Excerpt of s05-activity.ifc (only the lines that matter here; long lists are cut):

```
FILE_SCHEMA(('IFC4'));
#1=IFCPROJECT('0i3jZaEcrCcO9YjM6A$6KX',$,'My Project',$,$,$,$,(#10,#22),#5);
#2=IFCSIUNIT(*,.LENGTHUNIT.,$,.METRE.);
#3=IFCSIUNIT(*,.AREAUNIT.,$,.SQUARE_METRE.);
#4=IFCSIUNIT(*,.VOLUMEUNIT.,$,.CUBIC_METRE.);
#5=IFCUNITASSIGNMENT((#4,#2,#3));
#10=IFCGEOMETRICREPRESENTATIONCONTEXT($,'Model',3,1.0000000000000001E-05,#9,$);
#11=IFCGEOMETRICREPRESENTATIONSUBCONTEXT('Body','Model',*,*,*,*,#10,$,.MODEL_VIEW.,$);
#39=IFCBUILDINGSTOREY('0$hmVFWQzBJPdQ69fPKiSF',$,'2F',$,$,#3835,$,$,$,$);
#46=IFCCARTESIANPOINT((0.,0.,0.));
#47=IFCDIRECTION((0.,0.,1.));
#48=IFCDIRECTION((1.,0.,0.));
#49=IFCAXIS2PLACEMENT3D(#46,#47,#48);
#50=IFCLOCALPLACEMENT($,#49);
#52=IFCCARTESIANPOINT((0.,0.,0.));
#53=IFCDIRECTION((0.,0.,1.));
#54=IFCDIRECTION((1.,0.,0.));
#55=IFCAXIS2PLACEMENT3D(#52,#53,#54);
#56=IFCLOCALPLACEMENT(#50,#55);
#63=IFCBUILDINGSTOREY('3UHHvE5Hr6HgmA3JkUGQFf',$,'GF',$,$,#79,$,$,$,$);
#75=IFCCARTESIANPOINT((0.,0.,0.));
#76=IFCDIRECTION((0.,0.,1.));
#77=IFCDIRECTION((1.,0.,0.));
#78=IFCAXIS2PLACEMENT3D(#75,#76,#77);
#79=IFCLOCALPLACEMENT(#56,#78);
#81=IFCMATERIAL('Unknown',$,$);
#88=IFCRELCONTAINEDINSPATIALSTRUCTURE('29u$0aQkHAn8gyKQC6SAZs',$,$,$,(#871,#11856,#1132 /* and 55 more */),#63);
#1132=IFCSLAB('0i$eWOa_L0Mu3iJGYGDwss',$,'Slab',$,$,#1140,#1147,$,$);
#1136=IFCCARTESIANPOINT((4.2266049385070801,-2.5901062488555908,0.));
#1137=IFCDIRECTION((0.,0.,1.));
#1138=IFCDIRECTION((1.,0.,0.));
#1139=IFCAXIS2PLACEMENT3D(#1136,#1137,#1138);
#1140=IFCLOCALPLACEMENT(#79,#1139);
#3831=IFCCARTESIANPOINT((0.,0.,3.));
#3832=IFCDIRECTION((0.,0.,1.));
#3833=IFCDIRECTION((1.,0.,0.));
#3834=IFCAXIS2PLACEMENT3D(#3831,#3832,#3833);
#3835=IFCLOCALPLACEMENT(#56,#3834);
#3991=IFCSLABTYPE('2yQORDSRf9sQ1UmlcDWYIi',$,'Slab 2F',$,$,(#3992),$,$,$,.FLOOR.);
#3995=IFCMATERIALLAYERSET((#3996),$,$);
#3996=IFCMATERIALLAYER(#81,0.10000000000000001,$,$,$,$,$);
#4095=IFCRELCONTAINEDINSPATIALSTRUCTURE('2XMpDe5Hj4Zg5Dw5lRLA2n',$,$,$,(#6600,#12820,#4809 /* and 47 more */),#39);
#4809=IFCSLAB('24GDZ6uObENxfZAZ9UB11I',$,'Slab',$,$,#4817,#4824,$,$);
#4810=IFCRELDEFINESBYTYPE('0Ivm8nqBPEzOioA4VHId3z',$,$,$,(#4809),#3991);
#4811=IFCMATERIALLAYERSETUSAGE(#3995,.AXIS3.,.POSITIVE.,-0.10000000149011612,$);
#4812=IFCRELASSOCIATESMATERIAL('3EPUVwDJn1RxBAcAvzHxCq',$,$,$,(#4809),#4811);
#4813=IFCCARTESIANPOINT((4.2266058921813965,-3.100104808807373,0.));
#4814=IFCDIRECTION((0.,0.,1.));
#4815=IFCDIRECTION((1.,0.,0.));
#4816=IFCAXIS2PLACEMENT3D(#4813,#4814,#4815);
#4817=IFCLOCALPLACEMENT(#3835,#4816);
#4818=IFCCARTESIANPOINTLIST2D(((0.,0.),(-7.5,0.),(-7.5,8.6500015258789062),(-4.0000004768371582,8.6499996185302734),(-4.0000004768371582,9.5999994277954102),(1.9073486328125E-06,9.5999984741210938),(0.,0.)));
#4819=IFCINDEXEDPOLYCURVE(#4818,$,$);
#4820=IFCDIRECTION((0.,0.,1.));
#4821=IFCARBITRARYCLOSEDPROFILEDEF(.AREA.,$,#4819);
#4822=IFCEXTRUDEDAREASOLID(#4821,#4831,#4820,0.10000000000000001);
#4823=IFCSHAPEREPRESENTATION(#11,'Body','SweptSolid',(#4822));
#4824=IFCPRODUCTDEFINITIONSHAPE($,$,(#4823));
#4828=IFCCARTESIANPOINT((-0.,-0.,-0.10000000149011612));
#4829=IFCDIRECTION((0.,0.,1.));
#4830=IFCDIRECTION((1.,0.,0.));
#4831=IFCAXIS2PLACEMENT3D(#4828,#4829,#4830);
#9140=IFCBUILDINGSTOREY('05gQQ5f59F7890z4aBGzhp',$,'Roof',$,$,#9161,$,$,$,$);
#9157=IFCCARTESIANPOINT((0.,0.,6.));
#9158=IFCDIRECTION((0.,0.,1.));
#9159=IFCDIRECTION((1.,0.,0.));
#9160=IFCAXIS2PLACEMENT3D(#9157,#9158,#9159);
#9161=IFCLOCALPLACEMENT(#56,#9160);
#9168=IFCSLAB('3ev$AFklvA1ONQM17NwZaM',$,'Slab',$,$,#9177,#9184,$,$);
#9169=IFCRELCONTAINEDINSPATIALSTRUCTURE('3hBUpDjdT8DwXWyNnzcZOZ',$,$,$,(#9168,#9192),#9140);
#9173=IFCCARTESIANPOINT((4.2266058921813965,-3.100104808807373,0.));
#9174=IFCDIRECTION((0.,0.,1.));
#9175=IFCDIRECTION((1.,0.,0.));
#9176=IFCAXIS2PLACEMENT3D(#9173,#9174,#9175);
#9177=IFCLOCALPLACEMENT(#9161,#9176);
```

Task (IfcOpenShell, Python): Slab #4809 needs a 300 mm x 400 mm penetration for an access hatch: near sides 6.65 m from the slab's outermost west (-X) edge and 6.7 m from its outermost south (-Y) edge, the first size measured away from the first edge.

```python
import numpy as np
import ifcopenshell
import ifcopenshell.api.feature
import ifcopenshell.api.geometry
import ifcopenshell.api.root
import ifcopenshell.geom
import ifcopenshell.util.placement
import ifcopenshell.util.representation
import ifcopenshell.util.shape
import ifcopenshell.util.unit

model = ifcopenshell.open("s05-activity.ifc")
unit_scale = ifcopenshell.util.unit.calculate_unit_scale(model)
settings = ifcopenshell.geom.settings()


def volume(element):
    """Net volume in cubic metres, openings subtracted."""
    shape = ifcopenshell.geom.create_shape(settings, element)
    return ifcopenshell.util.shape.get_volume(shape.geometry)


slab = model.by_guid("24GDZ6uObENxfZAZ9UB11I")
before = volume(slab)

# Extent in the slab's own axes, in metres. The edges named are its -X and -Y sides.
slab_shape = ifcopenshell.geom.create_shape(settings, slab)
vertices = ifcopenshell.util.shape.get_vertices(slab_shape.geometry)
x_min, y_min, bottom = vertices.min(axis=0)
top = vertices[:, 2].max()

opening = ifcopenshell.api.root.create_entity(model, ifc_class="IfcOpeningElement", name="Access hatch opening", predefined_type="OPENING")
context = ifcopenshell.util.representation.get_context(model, "Model", "Body", "MODEL_VIEW")
width, depth = 0.3, 0.4
outline = [(0.0, 0.0), (width, 0.0), (width, depth), (0.0, depth), (0.0, 0.0)]
# Overshoot both faces by 50 mm so the cut is clean.
shape = ifcopenshell.api.geometry.add_slab_representation(
    model, context=context, depth=top - bottom + 0.1, polyline=outline
)
ifcopenshell.api.geometry.assign_representation(model, product=opening, representation=shape)

matrix = ifcopenshell.util.placement.get_local_placement(slab.ObjectPlacement)
matrix[:, 3] = matrix @ np.append(np.array([x_min + 6.65, y_min + 6.7, bottom - 0.05]) / unit_scale, 1.0)
ifcopenshell.api.geometry.edit_object_placement(model, product=opening, matrix=matrix, is_si=False)
ifcopenshell.api.feature.add_feature(model, feature=opening, element=slab)

after = volume(slab)

print(f"slab volume {before:.3f} -> {after:.3f} m3")

model.write("s05-activity_rev.ifc")
```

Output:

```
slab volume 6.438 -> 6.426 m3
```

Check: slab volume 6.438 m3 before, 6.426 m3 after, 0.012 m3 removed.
